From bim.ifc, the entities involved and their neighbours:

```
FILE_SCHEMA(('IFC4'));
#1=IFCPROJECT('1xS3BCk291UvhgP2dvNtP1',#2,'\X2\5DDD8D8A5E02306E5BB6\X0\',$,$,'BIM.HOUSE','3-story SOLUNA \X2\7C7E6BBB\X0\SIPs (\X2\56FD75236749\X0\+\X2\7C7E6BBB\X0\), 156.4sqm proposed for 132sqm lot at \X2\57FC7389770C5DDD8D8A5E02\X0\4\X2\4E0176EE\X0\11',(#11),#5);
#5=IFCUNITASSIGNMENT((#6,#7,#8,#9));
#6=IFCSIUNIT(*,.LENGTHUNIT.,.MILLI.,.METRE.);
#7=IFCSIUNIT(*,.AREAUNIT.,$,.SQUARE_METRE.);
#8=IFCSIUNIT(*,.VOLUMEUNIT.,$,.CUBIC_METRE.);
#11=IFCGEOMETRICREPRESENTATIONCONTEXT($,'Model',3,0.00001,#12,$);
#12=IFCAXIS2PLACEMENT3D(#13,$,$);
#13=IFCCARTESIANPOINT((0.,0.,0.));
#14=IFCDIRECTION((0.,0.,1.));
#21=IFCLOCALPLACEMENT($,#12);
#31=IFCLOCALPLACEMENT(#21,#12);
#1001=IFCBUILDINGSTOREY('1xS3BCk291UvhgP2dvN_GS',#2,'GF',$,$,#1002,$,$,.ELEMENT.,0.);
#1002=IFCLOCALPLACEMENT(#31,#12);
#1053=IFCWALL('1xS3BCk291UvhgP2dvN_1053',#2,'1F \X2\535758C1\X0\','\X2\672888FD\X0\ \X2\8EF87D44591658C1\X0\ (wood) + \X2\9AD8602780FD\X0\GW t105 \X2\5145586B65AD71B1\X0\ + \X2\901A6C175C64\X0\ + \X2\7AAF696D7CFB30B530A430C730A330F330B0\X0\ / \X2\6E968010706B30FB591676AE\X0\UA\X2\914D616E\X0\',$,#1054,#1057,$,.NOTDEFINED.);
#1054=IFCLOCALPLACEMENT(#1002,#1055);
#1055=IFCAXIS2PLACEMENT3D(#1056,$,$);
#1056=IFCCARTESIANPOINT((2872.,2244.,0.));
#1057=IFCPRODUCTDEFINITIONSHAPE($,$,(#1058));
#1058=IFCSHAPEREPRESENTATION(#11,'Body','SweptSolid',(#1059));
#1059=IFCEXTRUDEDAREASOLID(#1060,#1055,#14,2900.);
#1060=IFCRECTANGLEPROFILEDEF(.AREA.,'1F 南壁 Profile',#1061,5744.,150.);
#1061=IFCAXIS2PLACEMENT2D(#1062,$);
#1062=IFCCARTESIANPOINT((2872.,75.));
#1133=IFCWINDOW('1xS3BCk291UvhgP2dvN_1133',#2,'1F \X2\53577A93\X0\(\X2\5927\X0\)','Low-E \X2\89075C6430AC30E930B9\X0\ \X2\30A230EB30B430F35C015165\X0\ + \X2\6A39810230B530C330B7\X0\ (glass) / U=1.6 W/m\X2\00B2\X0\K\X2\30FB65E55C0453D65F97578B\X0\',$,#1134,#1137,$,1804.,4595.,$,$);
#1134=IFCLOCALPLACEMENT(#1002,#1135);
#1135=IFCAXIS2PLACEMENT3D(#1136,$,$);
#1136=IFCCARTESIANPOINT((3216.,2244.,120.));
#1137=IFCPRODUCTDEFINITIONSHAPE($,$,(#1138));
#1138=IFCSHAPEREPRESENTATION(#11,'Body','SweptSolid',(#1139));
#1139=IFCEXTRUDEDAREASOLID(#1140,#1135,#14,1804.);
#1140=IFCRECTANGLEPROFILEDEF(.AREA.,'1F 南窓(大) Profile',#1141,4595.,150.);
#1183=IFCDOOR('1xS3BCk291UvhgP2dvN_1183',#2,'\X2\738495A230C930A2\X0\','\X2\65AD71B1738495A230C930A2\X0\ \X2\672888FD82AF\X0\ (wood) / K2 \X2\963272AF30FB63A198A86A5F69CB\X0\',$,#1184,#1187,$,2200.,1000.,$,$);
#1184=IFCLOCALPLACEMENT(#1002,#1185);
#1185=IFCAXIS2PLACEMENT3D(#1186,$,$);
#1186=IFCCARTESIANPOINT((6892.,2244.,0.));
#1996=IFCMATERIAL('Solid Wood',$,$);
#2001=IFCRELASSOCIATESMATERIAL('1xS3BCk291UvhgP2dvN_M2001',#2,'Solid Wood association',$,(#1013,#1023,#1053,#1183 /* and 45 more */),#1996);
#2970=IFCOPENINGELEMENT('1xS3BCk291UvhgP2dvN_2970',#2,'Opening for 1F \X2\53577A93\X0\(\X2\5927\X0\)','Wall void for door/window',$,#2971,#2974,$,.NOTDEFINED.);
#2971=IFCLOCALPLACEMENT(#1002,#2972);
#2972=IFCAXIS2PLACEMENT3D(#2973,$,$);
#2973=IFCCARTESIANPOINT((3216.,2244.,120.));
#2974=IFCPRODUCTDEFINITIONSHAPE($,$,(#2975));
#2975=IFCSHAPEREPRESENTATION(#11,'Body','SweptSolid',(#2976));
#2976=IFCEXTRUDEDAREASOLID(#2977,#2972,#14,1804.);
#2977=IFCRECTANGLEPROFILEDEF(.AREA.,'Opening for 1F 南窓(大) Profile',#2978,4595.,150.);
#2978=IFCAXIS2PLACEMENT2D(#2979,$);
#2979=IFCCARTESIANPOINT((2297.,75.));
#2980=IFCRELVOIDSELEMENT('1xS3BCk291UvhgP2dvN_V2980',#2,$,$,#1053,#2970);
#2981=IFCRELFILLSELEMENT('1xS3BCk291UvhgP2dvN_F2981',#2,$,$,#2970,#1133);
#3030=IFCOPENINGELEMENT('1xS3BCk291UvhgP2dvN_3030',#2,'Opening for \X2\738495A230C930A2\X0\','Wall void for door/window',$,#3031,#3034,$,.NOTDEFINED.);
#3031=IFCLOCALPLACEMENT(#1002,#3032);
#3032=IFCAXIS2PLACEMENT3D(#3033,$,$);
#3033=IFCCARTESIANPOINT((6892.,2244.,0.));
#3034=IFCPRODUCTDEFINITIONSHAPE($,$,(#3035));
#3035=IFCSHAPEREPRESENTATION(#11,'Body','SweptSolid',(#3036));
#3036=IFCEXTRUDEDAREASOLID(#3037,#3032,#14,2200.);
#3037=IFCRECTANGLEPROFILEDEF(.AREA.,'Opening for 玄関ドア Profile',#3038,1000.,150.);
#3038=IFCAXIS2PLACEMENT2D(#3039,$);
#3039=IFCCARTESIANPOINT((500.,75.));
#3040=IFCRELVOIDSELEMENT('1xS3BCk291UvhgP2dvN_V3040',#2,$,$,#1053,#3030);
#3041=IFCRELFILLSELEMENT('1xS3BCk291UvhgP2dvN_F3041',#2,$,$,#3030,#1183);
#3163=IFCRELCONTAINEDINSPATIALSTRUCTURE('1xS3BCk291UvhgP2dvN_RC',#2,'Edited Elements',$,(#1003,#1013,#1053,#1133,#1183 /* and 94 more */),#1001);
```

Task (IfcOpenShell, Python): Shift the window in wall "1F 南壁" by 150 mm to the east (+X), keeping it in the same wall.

```python
import ifcopenshell
import ifcopenshell.api.geometry
import ifcopenshell.util.placement

model = ifcopenshell.open("bim.ifc")

window = model.by_guid("1xS3BCk291UvhgP2dvN_1133")
opening = window.FillsVoids[0].RelatingOpeningElement
wall = opening.VoidsElements[0].RelatingBuildingElement

wall_matrix = ifcopenshell.util.placement.get_local_placement(wall.ObjectPlacement)
shift = wall_matrix[:3, 0] * 150.0
before = ifcopenshell.util.placement.get_local_placement(window.ObjectPlacement)[:3, 3].copy()

# The window is not placed relative to its opening, so move both.
for product in (opening, window):
    matrix = ifcopenshell.util.placement.get_local_placement(product.ObjectPlacement)
    matrix[:3, 3] += shift
    ifcopenshell.api.geometry.edit_object_placement(model, product=product, matrix=matrix, is_si=False)

after = ifcopenshell.util.placement.get_local_placement(window.ObjectPlacement)[:3, 3]
print("window moved by", (after - before).round(3) + 0.0)

model.write("bim-out.ifc")
```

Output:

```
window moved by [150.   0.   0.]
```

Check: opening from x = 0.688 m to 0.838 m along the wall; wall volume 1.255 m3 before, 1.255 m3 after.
